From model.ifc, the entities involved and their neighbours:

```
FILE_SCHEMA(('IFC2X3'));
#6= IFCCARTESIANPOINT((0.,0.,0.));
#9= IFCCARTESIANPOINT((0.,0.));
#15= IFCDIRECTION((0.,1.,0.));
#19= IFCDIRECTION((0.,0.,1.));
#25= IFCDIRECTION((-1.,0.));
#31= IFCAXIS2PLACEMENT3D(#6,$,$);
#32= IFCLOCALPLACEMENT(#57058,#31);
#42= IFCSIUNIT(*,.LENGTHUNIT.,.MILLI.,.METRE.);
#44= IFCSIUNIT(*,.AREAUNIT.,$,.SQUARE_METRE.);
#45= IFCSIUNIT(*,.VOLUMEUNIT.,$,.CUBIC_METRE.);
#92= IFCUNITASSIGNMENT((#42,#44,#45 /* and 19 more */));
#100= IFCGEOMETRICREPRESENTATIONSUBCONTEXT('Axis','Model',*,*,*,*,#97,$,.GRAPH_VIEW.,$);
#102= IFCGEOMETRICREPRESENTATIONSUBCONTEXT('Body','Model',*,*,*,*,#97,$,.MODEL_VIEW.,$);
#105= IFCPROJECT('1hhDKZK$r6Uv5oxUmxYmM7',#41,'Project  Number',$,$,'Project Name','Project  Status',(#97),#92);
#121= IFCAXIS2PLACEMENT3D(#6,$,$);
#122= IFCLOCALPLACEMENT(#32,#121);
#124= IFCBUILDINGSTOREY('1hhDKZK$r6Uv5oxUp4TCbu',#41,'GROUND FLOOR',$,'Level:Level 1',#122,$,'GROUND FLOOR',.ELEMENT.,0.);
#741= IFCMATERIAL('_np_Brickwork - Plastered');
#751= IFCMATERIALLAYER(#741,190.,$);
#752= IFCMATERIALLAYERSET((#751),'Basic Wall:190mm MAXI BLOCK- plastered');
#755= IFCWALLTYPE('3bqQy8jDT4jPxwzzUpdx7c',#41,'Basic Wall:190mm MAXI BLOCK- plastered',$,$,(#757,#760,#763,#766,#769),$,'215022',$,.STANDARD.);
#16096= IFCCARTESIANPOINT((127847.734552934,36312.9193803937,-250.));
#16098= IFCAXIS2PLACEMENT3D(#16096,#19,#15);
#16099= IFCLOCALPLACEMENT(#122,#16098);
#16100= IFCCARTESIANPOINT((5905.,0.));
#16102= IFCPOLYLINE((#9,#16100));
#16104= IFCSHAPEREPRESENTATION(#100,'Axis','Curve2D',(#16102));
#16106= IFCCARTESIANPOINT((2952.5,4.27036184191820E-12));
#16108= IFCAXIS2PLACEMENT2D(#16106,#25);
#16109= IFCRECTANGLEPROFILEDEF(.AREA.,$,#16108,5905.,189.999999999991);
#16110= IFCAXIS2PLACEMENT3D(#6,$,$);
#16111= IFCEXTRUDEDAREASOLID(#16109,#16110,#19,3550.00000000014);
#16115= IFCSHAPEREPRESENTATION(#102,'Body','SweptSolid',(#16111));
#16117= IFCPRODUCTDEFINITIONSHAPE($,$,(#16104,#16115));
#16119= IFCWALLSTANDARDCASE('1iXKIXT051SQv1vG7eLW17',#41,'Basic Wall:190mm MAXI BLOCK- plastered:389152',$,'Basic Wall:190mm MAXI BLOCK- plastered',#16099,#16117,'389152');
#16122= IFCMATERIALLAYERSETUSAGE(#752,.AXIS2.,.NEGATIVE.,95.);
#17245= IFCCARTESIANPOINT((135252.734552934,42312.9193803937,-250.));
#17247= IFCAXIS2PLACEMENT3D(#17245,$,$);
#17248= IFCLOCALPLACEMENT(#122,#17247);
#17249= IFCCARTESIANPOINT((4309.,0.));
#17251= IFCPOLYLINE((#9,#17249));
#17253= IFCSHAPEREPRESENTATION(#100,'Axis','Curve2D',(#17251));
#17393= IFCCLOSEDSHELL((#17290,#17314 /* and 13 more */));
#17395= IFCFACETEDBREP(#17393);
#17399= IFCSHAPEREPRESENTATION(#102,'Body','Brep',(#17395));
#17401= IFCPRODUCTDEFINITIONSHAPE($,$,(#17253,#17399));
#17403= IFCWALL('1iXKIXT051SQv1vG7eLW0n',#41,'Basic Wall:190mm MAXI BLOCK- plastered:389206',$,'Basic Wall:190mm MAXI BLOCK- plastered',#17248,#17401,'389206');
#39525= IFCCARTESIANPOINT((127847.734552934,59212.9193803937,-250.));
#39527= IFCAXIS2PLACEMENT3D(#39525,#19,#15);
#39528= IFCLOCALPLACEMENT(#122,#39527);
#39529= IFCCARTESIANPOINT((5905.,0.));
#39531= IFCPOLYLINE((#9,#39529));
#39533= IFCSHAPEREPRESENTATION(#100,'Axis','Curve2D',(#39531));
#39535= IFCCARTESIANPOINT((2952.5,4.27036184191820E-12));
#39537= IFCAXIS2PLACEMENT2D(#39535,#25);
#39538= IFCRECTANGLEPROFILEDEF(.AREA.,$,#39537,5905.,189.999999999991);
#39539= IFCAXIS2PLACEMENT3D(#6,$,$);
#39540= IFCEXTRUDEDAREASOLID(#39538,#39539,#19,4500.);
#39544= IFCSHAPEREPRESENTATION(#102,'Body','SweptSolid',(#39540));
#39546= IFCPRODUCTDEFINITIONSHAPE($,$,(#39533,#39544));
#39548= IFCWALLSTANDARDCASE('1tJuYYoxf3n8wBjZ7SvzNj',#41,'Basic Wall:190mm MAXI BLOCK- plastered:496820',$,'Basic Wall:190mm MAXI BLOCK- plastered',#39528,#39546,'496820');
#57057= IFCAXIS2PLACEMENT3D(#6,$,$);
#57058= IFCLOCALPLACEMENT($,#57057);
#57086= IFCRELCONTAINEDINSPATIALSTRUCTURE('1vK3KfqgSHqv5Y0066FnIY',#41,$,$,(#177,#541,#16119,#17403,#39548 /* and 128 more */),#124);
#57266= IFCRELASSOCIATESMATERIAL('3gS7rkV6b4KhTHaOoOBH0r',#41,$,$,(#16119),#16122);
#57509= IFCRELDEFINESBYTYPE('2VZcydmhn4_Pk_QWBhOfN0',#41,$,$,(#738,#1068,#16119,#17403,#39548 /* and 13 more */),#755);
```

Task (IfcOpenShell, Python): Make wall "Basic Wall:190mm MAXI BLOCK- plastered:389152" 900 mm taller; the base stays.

```python
import ifcopenshell
import ifcopenshell.geom
import ifcopenshell.util.representation
import ifcopenshell.util.shape

model = ifcopenshell.open("model.ifc")
settings = ifcopenshell.geom.settings()


def volume(element):
    """Net volume in cubic metres, openings subtracted."""
    shape = ifcopenshell.geom.create_shape(settings, element)
    return ifcopenshell.util.shape.get_volume(shape.geometry)


wall = model.by_guid("1iXKIXT051SQv1vG7eLW17")
before = volume(wall)

body = ifcopenshell.util.representation.get_representation(wall, "Model", "Body")
solid = body.Items[0]
old_height = solid.Depth
solid.Depth += 900.0
after = volume(wall)

print(f"height {old_height:g} -> {solid.Depth:g}, volume {before:.3f} -> {after:.3f} m3")

model.write("model_edited.ifc")
```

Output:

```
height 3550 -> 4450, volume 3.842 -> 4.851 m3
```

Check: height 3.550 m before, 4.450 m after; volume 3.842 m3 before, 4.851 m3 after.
